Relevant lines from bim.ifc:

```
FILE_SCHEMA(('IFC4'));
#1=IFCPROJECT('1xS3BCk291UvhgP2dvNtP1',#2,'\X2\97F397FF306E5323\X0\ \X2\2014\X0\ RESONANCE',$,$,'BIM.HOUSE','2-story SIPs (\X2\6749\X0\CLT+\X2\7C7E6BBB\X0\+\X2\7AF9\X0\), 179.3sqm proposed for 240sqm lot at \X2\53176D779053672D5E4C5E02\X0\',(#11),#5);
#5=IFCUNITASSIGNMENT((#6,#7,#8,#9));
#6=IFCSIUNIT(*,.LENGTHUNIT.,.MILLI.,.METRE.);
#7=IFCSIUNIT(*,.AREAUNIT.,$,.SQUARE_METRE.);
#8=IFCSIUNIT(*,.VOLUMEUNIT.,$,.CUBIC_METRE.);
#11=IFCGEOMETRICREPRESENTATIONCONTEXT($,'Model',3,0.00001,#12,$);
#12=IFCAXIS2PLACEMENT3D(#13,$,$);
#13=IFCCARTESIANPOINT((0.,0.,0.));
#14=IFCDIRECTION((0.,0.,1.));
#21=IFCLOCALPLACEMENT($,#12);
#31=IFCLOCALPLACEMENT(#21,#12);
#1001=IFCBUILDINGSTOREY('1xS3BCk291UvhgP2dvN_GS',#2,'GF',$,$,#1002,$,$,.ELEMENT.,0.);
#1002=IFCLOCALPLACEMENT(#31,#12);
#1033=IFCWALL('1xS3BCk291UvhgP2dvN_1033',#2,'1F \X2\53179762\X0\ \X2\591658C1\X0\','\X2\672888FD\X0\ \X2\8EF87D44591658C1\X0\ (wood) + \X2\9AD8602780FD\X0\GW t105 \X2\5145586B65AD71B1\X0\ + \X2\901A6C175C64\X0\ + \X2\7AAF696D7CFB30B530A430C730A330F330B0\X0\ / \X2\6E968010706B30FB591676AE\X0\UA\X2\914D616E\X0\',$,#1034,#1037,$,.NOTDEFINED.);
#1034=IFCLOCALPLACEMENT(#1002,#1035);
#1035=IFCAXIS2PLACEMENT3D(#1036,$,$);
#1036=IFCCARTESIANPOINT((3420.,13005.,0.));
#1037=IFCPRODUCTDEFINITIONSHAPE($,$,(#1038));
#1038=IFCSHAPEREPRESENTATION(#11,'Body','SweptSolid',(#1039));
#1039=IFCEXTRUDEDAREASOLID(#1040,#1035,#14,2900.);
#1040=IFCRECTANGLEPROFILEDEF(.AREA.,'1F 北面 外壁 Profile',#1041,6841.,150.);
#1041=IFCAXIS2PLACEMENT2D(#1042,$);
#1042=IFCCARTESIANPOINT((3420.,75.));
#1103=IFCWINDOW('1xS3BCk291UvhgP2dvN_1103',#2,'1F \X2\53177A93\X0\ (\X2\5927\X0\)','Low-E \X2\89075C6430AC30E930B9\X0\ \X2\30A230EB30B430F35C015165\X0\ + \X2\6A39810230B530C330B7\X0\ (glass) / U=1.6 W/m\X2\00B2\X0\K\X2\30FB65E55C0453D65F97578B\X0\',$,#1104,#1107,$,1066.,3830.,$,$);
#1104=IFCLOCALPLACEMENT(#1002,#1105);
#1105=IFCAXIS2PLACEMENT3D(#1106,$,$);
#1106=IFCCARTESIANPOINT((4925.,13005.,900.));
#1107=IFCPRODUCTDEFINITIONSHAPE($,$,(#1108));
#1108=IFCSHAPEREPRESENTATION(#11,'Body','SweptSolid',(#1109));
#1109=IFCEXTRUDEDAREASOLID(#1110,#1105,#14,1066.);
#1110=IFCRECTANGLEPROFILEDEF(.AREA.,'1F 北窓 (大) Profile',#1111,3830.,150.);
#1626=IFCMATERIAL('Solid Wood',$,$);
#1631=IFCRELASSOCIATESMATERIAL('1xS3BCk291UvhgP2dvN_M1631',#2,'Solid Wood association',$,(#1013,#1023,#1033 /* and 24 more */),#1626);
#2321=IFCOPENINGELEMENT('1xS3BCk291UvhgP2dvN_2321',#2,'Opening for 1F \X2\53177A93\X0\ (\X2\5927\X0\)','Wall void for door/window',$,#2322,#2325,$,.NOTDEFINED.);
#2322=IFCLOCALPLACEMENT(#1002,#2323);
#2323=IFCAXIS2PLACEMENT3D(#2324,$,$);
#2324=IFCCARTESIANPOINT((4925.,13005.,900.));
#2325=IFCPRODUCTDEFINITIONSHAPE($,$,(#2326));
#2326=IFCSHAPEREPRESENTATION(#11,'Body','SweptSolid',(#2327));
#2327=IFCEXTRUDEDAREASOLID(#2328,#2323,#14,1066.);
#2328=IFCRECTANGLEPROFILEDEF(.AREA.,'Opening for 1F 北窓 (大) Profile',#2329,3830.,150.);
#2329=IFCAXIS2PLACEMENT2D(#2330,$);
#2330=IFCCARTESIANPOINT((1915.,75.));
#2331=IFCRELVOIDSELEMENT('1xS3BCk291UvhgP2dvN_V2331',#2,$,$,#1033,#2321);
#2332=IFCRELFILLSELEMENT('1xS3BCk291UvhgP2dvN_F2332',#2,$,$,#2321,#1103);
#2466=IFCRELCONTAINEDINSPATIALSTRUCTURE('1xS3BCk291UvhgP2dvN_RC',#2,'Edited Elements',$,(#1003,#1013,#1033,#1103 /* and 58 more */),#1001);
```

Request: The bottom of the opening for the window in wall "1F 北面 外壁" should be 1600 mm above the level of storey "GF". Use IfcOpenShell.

```python
import numpy as np
import ifcopenshell
import ifcopenshell.api.geometry
import ifcopenshell.geom
import ifcopenshell.util.element
import ifcopenshell.util.placement
import ifcopenshell.util.shape
import ifcopenshell.util.unit

model = ifcopenshell.open("bim.ifc")
unit_scale = ifcopenshell.util.unit.calculate_unit_scale(model)

window = model.by_guid("1xS3BCk291UvhgP2dvN_1103")
opening = window.FillsVoids[0].RelatingOpeningElement
storey = ifcopenshell.util.element.get_container(window, ifc_class="IfcBuildingStorey")
level = ifcopenshell.util.placement.get_local_placement(storey.ObjectPlacement)[2, 3]

# The opening's origin need not be at the sill, so measure its lowest point.
shape = ifcopenshell.geom.create_shape(ifcopenshell.geom.settings(), opening)
bottom = ifcopenshell.util.shape.get_shape_bottom_elevation(shape, shape.geometry) / unit_scale
dz = level + 1.6 / unit_scale - bottom

shift = np.array([0.0, 0.0, dz])
# The window is not placed relative to its opening, so move both.
for product in (opening, window):
    matrix = ifcopenshell.util.placement.get_local_placement(product.ObjectPlacement)
    matrix[:3, 3] += shift
    ifcopenshell.api.geometry.edit_object_placement(model, product=product, matrix=matrix, is_si=False)

print(f"moved by {dz * unit_scale:+.3f} m")

model.write("bim-out.ifc")
```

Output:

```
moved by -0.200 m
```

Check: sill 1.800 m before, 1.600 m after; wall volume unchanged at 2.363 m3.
